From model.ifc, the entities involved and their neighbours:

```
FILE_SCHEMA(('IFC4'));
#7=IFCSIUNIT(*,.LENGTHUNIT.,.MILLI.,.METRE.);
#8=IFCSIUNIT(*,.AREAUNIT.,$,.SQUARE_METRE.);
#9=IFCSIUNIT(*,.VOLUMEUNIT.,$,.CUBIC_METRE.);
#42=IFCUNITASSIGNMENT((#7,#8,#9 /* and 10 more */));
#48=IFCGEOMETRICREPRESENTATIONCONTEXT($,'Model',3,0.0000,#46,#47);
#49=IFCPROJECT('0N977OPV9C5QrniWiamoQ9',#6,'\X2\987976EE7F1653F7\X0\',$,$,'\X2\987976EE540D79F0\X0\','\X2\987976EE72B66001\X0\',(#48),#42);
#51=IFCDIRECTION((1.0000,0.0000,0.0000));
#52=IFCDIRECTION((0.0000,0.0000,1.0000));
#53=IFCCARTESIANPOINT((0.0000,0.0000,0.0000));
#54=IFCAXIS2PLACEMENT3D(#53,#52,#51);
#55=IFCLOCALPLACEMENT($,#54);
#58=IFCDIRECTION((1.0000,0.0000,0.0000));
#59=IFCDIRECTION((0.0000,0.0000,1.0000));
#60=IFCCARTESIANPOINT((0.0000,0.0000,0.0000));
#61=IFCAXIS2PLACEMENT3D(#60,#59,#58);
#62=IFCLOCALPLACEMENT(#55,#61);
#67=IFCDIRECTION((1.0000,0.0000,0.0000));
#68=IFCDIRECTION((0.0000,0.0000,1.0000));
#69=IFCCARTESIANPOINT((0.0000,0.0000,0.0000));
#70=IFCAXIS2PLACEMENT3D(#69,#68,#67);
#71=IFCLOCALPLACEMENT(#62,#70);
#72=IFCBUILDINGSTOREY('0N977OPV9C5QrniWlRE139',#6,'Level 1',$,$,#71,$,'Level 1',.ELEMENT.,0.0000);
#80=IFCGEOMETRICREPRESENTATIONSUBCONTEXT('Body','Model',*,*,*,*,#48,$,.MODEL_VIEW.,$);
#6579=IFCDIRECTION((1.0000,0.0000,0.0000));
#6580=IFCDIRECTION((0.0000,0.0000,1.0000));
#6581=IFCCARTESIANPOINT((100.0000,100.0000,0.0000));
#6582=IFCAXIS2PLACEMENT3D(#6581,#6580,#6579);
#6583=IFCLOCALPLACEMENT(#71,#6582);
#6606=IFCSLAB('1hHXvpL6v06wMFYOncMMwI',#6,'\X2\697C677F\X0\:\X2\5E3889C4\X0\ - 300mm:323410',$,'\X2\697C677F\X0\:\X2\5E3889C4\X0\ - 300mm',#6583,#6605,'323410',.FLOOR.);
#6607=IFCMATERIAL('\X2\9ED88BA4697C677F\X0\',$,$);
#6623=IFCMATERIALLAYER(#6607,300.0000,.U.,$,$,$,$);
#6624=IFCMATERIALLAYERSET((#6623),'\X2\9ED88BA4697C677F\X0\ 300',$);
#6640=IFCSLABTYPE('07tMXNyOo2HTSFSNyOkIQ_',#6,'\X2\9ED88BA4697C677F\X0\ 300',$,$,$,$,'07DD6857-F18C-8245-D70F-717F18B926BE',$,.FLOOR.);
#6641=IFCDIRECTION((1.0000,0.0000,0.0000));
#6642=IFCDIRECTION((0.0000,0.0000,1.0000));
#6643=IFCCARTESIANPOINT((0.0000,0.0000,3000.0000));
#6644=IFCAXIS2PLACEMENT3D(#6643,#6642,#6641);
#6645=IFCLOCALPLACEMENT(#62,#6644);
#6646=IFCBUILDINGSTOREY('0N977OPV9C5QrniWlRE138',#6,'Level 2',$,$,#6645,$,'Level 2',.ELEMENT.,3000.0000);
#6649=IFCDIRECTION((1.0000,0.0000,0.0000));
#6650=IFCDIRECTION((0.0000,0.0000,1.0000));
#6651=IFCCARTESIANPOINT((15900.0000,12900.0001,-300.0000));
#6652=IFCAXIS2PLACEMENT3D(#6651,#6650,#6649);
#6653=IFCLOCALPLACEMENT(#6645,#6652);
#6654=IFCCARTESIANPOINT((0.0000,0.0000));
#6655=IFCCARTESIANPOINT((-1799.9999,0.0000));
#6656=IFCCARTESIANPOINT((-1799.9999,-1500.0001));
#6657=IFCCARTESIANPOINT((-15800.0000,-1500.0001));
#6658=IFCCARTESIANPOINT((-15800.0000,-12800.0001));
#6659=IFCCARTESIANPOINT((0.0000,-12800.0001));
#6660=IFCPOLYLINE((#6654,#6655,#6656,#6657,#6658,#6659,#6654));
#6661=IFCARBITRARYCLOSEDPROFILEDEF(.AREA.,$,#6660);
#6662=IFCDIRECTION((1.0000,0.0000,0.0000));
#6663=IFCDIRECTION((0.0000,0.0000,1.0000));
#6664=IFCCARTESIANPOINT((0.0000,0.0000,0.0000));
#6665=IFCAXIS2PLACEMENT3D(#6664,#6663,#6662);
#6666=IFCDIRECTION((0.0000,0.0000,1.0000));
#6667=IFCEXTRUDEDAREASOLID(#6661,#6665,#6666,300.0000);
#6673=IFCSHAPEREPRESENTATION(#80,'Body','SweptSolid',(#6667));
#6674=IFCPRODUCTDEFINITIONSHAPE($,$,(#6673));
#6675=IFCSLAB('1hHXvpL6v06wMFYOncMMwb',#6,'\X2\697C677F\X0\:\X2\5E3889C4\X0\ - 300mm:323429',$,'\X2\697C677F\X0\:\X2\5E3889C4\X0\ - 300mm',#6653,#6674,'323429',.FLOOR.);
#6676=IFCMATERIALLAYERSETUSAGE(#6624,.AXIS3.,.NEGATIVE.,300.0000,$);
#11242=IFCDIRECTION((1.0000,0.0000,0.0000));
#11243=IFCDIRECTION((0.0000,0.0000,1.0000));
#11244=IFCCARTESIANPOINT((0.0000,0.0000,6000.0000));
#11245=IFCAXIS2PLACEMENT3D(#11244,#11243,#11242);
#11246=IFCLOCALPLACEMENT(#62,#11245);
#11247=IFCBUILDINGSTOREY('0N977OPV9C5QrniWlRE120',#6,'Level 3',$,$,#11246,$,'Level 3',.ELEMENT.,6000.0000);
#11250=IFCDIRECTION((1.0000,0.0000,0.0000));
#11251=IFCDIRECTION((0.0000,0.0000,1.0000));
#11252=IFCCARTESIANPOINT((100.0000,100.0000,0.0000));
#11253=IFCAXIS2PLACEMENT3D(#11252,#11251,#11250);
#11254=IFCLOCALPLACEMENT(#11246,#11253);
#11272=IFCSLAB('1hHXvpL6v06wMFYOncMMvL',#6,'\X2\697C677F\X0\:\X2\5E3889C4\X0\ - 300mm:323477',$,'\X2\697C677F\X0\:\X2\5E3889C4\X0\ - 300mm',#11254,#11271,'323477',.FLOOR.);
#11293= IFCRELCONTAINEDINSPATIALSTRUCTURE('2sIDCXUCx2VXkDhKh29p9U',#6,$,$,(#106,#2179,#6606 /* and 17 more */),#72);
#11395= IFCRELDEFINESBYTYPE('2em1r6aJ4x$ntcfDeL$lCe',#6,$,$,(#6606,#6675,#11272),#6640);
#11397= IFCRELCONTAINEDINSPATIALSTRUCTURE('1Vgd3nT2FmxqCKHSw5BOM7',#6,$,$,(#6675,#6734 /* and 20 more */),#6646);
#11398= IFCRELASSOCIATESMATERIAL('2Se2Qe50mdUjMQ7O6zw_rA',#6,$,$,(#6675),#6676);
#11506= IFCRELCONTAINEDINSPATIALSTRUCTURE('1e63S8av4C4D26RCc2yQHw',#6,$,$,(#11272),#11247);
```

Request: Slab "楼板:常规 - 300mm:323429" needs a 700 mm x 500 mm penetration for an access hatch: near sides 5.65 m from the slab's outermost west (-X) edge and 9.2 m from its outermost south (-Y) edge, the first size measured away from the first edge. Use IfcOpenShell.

```python
import numpy as np
import ifcopenshell
import ifcopenshell.api.feature
import ifcopenshell.api.geometry
import ifcopenshell.api.root
import ifcopenshell.geom
import ifcopenshell.util.placement
import ifcopenshell.util.representation
import ifcopenshell.util.shape
import ifcopenshell.util.unit

model = ifcopenshell.open("model.ifc")
unit_scale = ifcopenshell.util.unit.calculate_unit_scale(model)
settings = ifcopenshell.geom.settings()


def volume(element):
    """Net volume in cubic metres, openings subtracted."""
    shape = ifcopenshell.geom.create_shape(settings, element)
    return ifcopenshell.util.shape.get_volume(shape.geometry)


slab = model.by_guid("1hHXvpL6v06wMFYOncMMwb")
before = volume(slab)

# Extent in the slab's own axes, in metres. The edges named are its -X and -Y sides.
slab_shape = ifcopenshell.geom.create_shape(settings, slab)
vertices = ifcopenshell.util.shape.get_vertices(slab_shape.geometry)
x_min, y_min, bottom = vertices.min(axis=0)
top = vertices[:, 2].max()

opening = ifcopenshell.api.root.create_entity(model, ifc_class="IfcOpeningElement", name="Access hatch opening", predefined_type="OPENING")
context = ifcopenshell.util.representation.get_context(model, "Model", "Body", "MODEL_VIEW")
width, depth = 0.7, 0.5
outline = [(0.0, 0.0), (width, 0.0), (width, depth), (0.0, depth), (0.0, 0.0)]
# Overshoot both faces by 50 mm so the cut is clean.
shape = ifcopenshell.api.geometry.add_slab_representation(
    model, context=context, depth=top - bottom + 0.1, polyline=outline
)
ifcopenshell.api.geometry.assign_representation(model, product=opening, representation=shape)

matrix = ifcopenshell.util.placement.get_local_placement(slab.ObjectPlacement)
matrix[:, 3] = matrix @ np.append(np.array([x_min + 5.65, y_min + 9.2, bottom - 0.05]) / unit_scale, 1.0)
ifcopenshell.api.geometry.edit_object_placement(model, product=opening, matrix=matrix, is_si=False)
ifcopenshell.api.feature.add_feature(model, feature=opening, element=slab)

after = volume(slab)

print(f"slab volume {before:.3f} -> {after:.3f} m3")

model.write("model-out.ifc")
```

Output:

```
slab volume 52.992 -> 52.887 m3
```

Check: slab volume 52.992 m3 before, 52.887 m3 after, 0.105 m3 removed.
